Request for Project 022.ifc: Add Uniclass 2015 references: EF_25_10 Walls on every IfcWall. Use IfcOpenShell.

First a look at what the model holds.

```python
import ifcopenshell

model = ifcopenshell.open("Project 022.ifc")
print(model.schema)
print("classifications:", [c.Name for c in model.by_type("IfcClassification")])
for ifc_class in ("IfcDoor", "IfcRoof", "IfcStair", "IfcWall", "IfcWindow"):
    print(ifc_class, len(model.by_type(ifc_class)))
```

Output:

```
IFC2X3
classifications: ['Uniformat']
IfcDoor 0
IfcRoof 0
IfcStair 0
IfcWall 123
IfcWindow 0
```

```python
import ifcopenshell
import ifcopenshell.api.classification

model = ifcopenshell.open("Project 022.ifc")

# IFC2X3 requires Source and Edition and has no link from the project to the system.
system = model.create_entity("IfcClassification", Source="NBS", Edition="2015", Name="Uniclass 2015")

codes = {
    "IfcWall": ("EF_25_10", "Walls"),
}
for ifc_class, (code, name) in codes.items():
    products = model.by_type(ifc_class)
    ifcopenshell.api.classification.add_reference(
        model, products=products, classification=system, identification=code, name=name
    )
    print(code, len(products))

model.write("Project 022_v2.ifc")
```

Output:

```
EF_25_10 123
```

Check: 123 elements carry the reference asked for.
